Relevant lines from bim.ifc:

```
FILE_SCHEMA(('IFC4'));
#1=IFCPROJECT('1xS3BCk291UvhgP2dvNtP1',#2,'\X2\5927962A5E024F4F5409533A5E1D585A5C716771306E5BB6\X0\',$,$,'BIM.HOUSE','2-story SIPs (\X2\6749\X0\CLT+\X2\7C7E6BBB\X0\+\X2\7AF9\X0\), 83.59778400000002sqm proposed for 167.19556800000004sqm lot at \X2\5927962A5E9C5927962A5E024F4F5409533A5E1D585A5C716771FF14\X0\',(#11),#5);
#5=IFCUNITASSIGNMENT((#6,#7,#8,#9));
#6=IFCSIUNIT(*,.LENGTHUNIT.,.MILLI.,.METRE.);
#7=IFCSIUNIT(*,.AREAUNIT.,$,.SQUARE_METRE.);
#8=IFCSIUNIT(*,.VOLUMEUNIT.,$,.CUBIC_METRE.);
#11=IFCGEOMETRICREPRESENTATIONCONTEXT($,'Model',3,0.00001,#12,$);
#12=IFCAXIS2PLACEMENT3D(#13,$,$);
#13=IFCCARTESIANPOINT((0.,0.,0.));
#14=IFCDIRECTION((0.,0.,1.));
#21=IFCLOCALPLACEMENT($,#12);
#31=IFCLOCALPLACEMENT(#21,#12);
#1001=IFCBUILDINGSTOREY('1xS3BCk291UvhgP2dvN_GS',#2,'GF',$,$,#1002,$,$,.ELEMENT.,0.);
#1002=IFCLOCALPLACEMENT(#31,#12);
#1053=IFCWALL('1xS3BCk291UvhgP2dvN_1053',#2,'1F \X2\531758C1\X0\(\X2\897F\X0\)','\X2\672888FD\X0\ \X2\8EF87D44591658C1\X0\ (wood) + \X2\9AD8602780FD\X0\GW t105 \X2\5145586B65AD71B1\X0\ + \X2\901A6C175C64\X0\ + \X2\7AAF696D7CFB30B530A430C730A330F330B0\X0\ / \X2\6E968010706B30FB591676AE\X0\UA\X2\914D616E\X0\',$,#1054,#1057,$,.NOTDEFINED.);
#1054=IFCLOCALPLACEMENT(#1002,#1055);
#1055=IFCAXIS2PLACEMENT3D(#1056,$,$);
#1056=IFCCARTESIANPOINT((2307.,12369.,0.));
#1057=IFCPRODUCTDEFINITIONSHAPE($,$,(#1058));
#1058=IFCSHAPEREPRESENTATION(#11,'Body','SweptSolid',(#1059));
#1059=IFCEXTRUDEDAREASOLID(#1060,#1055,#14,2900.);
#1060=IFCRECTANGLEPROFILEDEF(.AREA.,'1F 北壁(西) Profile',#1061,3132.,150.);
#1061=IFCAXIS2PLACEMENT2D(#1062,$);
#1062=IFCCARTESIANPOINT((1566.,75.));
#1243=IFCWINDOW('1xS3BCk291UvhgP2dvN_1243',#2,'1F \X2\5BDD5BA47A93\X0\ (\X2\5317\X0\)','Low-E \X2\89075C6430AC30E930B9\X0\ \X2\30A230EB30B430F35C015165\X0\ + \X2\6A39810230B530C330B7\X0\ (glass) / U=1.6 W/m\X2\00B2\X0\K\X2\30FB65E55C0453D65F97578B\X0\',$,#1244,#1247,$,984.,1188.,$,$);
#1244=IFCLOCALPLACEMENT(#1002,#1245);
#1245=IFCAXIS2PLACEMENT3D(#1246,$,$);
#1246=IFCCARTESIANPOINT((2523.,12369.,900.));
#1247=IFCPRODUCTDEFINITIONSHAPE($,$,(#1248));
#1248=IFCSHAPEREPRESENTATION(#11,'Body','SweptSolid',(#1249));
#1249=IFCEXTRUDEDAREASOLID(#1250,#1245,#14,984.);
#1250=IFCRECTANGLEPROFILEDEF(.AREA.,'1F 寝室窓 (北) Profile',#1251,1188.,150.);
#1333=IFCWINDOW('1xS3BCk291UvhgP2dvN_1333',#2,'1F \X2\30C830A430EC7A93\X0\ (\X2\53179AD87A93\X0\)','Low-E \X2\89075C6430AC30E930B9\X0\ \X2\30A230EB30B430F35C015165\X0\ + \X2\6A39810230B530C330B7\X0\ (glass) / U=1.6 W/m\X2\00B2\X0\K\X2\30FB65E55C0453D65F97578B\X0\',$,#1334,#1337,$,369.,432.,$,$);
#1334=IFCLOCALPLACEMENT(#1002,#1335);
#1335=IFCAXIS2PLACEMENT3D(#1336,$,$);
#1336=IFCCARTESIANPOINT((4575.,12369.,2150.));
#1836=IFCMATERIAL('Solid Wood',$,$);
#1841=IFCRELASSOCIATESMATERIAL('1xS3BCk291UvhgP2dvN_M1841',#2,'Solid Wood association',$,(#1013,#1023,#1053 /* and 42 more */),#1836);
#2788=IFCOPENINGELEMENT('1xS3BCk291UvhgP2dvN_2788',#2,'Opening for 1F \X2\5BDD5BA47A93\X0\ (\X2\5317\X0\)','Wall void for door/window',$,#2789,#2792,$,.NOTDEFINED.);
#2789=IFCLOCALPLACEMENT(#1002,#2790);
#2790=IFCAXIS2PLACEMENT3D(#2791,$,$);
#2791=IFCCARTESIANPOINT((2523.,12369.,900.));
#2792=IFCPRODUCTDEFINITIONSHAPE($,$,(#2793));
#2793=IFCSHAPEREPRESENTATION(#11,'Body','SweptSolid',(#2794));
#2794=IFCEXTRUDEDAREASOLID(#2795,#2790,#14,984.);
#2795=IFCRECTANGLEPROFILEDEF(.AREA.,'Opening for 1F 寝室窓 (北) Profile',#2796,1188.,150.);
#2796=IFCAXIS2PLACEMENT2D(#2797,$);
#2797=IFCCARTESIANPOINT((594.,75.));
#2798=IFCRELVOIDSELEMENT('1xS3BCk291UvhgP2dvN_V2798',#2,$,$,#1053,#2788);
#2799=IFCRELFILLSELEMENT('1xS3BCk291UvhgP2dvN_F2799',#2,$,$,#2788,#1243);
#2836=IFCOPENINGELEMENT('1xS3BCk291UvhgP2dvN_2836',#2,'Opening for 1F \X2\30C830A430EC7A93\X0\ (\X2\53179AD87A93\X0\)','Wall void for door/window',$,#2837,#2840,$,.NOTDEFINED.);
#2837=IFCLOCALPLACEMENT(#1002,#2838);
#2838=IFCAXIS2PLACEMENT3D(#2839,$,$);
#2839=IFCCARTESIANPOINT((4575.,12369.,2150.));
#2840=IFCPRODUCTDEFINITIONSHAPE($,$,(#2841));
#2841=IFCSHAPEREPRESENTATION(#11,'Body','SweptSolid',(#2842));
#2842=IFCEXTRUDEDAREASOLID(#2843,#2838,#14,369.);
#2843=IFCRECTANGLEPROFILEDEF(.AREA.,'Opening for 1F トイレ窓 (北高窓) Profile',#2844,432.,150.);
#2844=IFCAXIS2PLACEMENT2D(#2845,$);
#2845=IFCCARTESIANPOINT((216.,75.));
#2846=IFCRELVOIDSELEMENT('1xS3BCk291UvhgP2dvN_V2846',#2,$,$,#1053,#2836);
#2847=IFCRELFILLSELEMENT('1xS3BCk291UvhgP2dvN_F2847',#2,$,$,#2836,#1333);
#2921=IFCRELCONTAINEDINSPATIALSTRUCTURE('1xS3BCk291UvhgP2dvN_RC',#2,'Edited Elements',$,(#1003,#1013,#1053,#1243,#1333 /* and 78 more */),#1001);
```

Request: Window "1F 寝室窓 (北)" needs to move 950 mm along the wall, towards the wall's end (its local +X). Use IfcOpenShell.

```python
import ifcopenshell
import ifcopenshell.api.geometry
import ifcopenshell.util.placement
import ifcopenshell.util.unit

model = ifcopenshell.open("bim.ifc")
unit_scale = ifcopenshell.util.unit.calculate_unit_scale(model)

window = model.by_guid("1xS3BCk291UvhgP2dvN_1243")
opening = window.FillsVoids[0].RelatingOpeningElement
wall = opening.VoidsElements[0].RelatingBuildingElement

wall_matrix = ifcopenshell.util.placement.get_local_placement(wall.ObjectPlacement)
shift = wall_matrix[:3, 0] * 0.95 / unit_scale
before = ifcopenshell.util.placement.get_local_placement(window.ObjectPlacement)[:3, 3].copy()

# The window is not placed relative to its opening, so move both.
for product in (opening, window):
    matrix = ifcopenshell.util.placement.get_local_placement(product.ObjectPlacement)
    matrix[:3, 3] += shift
    ifcopenshell.api.geometry.edit_object_placement(model, product=product, matrix=matrix, is_si=False)

after = ifcopenshell.util.placement.get_local_placement(window.ObjectPlacement)[:3, 3]
print("window moved by", (after - before).round(3) + 0.0)

model.write("bim_updated.ifc")
```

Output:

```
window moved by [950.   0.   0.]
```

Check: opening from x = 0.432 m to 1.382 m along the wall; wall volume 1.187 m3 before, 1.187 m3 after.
